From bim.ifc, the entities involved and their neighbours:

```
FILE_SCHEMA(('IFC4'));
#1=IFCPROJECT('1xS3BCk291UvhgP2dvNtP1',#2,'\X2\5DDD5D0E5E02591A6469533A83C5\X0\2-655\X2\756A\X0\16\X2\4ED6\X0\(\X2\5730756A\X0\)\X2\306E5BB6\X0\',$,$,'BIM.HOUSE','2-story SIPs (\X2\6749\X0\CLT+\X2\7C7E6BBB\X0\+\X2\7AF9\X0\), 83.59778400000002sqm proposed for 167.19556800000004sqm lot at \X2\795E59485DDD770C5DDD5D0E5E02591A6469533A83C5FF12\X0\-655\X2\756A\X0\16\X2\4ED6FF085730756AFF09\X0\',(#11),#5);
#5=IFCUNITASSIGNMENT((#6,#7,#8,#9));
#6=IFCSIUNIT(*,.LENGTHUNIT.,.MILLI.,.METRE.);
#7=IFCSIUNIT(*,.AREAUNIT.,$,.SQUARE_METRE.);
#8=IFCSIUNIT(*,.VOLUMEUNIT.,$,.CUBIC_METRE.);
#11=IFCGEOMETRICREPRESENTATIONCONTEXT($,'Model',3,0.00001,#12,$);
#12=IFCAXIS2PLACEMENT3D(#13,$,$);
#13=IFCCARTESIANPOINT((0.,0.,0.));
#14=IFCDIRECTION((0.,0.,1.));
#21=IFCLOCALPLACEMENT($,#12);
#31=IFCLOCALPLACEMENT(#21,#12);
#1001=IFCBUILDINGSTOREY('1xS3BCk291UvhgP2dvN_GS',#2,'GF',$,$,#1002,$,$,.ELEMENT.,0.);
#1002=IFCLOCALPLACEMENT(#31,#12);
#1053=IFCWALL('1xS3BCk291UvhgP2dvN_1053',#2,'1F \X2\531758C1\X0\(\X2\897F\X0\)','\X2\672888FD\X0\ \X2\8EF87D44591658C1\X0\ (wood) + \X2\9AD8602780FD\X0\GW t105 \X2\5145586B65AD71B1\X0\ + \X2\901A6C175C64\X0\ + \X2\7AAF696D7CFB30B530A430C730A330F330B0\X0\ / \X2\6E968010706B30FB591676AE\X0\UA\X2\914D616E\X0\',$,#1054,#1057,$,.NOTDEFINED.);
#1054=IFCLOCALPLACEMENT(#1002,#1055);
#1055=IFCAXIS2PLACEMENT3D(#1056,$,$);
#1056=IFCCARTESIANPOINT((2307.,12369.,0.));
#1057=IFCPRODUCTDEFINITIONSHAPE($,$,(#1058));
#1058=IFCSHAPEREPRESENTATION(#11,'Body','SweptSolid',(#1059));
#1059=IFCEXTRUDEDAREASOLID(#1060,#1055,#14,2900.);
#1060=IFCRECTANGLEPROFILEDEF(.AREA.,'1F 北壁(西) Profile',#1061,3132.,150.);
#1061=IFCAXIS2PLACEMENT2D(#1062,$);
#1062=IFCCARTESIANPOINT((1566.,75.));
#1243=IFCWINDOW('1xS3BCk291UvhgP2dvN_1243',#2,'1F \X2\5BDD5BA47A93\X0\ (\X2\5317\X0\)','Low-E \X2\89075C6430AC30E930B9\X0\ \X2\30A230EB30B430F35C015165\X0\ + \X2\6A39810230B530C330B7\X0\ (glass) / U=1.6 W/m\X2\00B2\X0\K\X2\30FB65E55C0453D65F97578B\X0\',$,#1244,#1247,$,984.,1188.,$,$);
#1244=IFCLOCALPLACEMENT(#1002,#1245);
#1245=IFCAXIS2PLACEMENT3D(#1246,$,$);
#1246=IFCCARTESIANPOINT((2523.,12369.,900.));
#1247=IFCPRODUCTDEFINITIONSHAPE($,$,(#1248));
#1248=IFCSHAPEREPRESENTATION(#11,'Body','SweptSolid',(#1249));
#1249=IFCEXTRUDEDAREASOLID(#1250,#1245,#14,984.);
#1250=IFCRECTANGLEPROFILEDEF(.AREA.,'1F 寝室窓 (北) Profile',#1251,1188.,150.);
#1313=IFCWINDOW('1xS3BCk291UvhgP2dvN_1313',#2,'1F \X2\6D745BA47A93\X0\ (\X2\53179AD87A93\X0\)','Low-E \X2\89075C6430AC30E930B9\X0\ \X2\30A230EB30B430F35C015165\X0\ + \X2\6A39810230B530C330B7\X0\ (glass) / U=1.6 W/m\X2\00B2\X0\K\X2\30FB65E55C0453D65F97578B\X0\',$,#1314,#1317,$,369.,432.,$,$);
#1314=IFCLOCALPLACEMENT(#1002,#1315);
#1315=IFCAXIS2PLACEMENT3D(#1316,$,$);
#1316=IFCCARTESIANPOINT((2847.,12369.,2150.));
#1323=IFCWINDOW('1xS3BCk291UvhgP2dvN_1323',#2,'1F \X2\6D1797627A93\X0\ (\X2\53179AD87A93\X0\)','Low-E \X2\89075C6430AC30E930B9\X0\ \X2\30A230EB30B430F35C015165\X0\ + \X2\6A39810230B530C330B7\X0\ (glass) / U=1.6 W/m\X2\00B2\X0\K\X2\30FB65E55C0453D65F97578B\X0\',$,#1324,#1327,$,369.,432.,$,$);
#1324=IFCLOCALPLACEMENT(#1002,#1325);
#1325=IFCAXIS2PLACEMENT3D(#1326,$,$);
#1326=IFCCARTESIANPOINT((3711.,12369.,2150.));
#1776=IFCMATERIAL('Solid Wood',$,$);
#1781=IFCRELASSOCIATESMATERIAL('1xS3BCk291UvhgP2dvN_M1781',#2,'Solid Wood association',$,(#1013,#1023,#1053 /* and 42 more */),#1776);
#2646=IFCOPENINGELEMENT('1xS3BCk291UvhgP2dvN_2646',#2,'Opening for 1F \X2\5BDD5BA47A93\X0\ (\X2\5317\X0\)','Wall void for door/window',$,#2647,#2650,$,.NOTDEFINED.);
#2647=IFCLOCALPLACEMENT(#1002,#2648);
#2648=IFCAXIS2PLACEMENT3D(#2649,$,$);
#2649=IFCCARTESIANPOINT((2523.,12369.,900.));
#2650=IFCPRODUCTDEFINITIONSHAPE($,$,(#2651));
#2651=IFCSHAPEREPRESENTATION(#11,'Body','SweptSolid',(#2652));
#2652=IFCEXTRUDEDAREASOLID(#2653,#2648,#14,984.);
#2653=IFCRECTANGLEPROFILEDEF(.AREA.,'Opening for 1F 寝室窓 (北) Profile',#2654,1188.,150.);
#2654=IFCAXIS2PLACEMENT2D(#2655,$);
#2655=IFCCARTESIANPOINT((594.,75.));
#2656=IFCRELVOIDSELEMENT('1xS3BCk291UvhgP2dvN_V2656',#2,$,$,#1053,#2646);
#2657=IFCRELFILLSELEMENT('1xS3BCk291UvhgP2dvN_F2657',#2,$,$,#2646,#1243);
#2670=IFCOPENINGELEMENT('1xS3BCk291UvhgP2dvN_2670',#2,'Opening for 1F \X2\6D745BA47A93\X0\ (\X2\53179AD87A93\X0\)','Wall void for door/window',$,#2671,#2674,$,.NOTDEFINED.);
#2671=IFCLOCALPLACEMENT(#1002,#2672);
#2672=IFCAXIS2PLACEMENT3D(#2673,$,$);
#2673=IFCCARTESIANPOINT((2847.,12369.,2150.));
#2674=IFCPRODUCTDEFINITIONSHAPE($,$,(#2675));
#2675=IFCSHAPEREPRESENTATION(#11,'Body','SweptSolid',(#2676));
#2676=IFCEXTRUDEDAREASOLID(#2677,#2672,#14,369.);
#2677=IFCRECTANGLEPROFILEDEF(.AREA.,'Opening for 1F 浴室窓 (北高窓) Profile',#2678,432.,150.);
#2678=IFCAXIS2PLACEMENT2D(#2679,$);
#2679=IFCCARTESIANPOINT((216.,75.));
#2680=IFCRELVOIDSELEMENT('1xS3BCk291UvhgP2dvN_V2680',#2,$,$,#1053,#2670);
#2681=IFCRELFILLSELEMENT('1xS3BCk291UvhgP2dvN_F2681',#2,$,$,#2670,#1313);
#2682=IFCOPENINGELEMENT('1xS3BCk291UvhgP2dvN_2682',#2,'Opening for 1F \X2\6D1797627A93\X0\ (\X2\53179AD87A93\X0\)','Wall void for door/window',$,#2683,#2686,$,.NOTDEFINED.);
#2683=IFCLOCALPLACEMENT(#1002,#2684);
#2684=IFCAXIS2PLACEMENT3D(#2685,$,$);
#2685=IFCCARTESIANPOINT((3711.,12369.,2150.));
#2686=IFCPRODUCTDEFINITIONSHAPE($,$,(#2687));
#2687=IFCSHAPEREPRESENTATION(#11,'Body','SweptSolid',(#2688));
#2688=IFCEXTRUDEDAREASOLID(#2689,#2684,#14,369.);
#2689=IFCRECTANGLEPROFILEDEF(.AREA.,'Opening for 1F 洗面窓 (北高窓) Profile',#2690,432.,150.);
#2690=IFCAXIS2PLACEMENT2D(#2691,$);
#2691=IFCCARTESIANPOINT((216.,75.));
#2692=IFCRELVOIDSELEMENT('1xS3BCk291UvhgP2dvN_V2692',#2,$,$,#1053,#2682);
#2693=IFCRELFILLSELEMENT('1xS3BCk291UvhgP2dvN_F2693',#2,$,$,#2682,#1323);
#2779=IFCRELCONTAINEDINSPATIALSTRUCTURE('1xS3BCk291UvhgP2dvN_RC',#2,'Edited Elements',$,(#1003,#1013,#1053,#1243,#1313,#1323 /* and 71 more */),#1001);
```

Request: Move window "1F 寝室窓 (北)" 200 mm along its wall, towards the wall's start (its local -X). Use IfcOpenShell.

```python
import ifcopenshell
import ifcopenshell.api.geometry
import ifcopenshell.util.placement
import ifcopenshell.util.unit

model = ifcopenshell.open("bim.ifc")
unit_scale = ifcopenshell.util.unit.calculate_unit_scale(model)

window = model.by_guid("1xS3BCk291UvhgP2dvN_1243")
opening = window.FillsVoids[0].RelatingOpeningElement
wall = opening.VoidsElements[0].RelatingBuildingElement

wall_matrix = ifcopenshell.util.placement.get_local_placement(wall.ObjectPlacement)
shift = wall_matrix[:3, 0] * -0.2 / unit_scale
before = ifcopenshell.util.placement.get_local_placement(window.ObjectPlacement)[:3, 3].copy()

# The window is not placed relative to its opening, so move both.
for product in (opening, window):
    matrix = ifcopenshell.util.placement.get_local_placement(product.ObjectPlacement)
    matrix[:3, 3] += shift
    ifcopenshell.api.geometry.edit_object_placement(model, product=product, matrix=matrix, is_si=False)

after = ifcopenshell.util.placement.get_local_placement(window.ObjectPlacement)[:3, 3]
print("window moved by", (after - before).round(3) + 0.0)

model.write("bim_updated.ifc")
```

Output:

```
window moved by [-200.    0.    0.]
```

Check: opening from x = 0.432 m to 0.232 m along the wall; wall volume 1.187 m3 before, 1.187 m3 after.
